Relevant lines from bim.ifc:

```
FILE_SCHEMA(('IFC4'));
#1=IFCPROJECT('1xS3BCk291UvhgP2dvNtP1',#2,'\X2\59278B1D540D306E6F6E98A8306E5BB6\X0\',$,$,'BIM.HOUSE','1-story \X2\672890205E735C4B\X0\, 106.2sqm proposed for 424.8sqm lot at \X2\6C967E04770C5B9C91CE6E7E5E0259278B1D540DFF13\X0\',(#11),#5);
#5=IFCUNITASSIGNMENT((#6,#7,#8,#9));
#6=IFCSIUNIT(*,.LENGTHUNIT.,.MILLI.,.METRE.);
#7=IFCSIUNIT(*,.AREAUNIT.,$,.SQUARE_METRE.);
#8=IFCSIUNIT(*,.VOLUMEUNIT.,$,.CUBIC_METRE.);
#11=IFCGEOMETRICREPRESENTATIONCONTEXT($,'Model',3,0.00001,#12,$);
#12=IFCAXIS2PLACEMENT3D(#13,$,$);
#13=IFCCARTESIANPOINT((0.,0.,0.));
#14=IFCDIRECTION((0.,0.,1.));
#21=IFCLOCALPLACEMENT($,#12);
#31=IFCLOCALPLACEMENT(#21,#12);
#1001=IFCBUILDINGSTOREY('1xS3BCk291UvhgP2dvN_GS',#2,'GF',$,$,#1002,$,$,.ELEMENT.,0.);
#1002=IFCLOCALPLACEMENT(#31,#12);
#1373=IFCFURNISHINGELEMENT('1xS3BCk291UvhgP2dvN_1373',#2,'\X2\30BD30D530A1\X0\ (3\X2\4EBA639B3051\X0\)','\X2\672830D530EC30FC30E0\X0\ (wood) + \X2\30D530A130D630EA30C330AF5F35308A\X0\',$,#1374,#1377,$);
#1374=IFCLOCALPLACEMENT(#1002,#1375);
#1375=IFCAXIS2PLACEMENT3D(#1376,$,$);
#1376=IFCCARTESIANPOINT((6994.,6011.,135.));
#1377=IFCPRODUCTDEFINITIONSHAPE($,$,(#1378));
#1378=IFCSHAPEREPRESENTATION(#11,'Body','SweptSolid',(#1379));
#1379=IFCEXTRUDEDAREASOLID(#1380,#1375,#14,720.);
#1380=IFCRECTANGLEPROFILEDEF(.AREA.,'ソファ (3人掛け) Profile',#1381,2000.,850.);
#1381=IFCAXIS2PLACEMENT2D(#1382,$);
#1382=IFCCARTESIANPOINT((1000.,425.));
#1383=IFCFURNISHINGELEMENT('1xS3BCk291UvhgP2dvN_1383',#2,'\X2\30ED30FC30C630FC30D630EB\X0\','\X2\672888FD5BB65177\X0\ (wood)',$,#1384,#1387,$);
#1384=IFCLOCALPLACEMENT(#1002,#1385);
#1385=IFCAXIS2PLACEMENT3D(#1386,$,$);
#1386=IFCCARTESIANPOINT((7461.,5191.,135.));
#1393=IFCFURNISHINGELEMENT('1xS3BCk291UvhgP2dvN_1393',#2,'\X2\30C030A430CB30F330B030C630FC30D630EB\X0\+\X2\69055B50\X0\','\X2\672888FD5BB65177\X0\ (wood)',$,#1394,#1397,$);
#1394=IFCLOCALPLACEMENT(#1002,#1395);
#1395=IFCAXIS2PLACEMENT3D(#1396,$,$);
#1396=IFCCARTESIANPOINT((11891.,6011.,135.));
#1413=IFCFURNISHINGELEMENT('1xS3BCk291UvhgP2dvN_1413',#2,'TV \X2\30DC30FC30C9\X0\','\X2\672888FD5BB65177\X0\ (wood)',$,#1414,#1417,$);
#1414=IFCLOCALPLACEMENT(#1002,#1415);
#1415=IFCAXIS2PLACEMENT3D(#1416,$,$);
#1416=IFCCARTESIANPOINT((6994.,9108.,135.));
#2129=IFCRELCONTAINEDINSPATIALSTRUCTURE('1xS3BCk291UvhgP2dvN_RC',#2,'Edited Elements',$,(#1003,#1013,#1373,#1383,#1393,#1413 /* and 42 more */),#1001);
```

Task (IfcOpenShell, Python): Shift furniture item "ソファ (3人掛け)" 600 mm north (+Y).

```python
import ifcopenshell
import ifcopenshell.api.geometry
import ifcopenshell.util.placement
import ifcopenshell.util.unit

model = ifcopenshell.open("bim.ifc")
unit_scale = ifcopenshell.util.unit.calculate_unit_scale(model)

item = model.by_id(1373)
matrix = ifcopenshell.util.placement.get_local_placement(item.ObjectPlacement)
matrix[1, 3] += 0.6 / unit_scale
ifcopenshell.api.geometry.edit_object_placement(model, product=item, matrix=matrix, is_si=False)

print(ifcopenshell.util.placement.get_local_placement(item.ObjectPlacement).round(3) + 0.0)

model.write("bim_edited.ifc")
```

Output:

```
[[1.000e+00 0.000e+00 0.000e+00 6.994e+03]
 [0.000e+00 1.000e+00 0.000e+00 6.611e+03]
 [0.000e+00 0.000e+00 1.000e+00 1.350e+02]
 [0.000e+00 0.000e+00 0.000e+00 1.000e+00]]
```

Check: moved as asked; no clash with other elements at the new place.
